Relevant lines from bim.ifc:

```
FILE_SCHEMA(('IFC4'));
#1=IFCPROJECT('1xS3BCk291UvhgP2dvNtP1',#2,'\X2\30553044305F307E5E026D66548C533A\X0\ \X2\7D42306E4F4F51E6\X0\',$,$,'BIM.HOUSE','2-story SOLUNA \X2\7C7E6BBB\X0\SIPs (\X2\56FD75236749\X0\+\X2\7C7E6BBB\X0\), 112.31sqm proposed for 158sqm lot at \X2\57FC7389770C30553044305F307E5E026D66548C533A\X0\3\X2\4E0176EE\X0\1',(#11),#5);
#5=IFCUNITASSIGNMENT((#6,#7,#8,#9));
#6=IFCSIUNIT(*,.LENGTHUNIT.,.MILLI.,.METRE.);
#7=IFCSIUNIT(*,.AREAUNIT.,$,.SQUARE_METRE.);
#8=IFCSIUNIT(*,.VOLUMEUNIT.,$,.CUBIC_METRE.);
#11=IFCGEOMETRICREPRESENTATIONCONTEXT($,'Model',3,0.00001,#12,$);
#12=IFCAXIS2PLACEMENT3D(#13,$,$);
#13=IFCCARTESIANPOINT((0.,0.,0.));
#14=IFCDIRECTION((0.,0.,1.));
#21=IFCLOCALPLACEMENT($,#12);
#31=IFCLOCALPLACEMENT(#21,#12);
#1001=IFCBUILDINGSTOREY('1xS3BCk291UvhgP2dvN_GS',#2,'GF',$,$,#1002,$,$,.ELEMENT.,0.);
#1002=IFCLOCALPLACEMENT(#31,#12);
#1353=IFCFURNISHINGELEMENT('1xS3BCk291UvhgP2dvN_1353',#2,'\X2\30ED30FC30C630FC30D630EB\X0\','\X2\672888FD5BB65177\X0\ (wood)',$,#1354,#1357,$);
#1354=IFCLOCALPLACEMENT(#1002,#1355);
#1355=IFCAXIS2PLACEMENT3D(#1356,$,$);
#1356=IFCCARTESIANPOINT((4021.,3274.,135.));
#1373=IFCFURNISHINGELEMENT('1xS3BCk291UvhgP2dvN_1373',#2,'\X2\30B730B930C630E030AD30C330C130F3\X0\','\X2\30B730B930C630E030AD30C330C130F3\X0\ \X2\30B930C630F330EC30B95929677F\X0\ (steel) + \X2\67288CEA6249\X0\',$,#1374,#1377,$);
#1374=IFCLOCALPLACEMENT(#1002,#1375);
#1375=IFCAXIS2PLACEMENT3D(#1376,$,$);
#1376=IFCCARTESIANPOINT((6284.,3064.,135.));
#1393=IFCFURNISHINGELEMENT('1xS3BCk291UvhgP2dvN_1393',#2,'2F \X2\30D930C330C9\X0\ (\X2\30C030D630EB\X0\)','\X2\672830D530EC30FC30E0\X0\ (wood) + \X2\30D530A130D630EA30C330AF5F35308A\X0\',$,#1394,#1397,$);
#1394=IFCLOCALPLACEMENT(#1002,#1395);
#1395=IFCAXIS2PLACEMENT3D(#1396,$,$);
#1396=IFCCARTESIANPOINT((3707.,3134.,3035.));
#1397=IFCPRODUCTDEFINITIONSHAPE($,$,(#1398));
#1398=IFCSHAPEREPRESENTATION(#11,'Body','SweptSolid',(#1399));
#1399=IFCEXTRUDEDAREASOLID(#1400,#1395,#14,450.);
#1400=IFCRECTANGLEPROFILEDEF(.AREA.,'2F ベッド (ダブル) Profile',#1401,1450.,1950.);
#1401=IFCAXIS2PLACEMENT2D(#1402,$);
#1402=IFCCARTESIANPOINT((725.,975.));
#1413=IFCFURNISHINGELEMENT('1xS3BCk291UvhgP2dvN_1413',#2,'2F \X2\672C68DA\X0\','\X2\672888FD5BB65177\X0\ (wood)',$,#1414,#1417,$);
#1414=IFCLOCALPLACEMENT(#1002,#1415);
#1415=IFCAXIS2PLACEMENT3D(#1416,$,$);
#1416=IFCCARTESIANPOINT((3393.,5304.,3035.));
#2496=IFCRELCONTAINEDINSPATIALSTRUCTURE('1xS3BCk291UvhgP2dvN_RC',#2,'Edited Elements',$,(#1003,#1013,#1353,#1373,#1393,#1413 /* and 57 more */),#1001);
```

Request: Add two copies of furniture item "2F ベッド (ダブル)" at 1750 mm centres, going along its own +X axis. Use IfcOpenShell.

```python
import ifcopenshell
import ifcopenshell.api.geometry
import ifcopenshell.api.root
import ifcopenshell.util.element
import ifcopenshell.util.placement
import ifcopenshell.util.unit

model = ifcopenshell.open("bim.ifc")
unit_scale = ifcopenshell.util.unit.calculate_unit_scale(model)


def reuse_history(source, copy):
    """copy_class also copies each property set's owner history, people and application; keep the originals."""
    for rel in copy.IsDefinedBy:
        if rel.is_a("IfcRelDefinesByProperties") and (history := rel.RelatingPropertyDefinition.OwnerHistory):
            rel.RelatingPropertyDefinition.OwnerHistory = source.OwnerHistory
            ifcopenshell.util.element.remove_deep2(model, history)


source = model.by_guid("1xS3BCk291UvhgP2dvN_1393")
base = ifcopenshell.util.placement.get_local_placement(source.ObjectPlacement)
step = base[:3, 0] * 1.75 / unit_scale

for i in range(1, 3):
    copy = ifcopenshell.api.root.copy_class(model, product=source)
    copy.Representation = ifcopenshell.util.element.copy_deep(
        model, source.Representation, exclude=["IfcGeometricRepresentationContext", "IfcRepresentationMap"]
    )
    reuse_history(source, copy)
    matrix = base.copy()
    matrix[:3, 3] += i * step
    print("added at", matrix[:3, 3].round(3) + 0.0)
    ifcopenshell.api.geometry.edit_object_placement(model, product=copy, matrix=matrix, is_si=False)

model.write("bim_updated.ifc")
```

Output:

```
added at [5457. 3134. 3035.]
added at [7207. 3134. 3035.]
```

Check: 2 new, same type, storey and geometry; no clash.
